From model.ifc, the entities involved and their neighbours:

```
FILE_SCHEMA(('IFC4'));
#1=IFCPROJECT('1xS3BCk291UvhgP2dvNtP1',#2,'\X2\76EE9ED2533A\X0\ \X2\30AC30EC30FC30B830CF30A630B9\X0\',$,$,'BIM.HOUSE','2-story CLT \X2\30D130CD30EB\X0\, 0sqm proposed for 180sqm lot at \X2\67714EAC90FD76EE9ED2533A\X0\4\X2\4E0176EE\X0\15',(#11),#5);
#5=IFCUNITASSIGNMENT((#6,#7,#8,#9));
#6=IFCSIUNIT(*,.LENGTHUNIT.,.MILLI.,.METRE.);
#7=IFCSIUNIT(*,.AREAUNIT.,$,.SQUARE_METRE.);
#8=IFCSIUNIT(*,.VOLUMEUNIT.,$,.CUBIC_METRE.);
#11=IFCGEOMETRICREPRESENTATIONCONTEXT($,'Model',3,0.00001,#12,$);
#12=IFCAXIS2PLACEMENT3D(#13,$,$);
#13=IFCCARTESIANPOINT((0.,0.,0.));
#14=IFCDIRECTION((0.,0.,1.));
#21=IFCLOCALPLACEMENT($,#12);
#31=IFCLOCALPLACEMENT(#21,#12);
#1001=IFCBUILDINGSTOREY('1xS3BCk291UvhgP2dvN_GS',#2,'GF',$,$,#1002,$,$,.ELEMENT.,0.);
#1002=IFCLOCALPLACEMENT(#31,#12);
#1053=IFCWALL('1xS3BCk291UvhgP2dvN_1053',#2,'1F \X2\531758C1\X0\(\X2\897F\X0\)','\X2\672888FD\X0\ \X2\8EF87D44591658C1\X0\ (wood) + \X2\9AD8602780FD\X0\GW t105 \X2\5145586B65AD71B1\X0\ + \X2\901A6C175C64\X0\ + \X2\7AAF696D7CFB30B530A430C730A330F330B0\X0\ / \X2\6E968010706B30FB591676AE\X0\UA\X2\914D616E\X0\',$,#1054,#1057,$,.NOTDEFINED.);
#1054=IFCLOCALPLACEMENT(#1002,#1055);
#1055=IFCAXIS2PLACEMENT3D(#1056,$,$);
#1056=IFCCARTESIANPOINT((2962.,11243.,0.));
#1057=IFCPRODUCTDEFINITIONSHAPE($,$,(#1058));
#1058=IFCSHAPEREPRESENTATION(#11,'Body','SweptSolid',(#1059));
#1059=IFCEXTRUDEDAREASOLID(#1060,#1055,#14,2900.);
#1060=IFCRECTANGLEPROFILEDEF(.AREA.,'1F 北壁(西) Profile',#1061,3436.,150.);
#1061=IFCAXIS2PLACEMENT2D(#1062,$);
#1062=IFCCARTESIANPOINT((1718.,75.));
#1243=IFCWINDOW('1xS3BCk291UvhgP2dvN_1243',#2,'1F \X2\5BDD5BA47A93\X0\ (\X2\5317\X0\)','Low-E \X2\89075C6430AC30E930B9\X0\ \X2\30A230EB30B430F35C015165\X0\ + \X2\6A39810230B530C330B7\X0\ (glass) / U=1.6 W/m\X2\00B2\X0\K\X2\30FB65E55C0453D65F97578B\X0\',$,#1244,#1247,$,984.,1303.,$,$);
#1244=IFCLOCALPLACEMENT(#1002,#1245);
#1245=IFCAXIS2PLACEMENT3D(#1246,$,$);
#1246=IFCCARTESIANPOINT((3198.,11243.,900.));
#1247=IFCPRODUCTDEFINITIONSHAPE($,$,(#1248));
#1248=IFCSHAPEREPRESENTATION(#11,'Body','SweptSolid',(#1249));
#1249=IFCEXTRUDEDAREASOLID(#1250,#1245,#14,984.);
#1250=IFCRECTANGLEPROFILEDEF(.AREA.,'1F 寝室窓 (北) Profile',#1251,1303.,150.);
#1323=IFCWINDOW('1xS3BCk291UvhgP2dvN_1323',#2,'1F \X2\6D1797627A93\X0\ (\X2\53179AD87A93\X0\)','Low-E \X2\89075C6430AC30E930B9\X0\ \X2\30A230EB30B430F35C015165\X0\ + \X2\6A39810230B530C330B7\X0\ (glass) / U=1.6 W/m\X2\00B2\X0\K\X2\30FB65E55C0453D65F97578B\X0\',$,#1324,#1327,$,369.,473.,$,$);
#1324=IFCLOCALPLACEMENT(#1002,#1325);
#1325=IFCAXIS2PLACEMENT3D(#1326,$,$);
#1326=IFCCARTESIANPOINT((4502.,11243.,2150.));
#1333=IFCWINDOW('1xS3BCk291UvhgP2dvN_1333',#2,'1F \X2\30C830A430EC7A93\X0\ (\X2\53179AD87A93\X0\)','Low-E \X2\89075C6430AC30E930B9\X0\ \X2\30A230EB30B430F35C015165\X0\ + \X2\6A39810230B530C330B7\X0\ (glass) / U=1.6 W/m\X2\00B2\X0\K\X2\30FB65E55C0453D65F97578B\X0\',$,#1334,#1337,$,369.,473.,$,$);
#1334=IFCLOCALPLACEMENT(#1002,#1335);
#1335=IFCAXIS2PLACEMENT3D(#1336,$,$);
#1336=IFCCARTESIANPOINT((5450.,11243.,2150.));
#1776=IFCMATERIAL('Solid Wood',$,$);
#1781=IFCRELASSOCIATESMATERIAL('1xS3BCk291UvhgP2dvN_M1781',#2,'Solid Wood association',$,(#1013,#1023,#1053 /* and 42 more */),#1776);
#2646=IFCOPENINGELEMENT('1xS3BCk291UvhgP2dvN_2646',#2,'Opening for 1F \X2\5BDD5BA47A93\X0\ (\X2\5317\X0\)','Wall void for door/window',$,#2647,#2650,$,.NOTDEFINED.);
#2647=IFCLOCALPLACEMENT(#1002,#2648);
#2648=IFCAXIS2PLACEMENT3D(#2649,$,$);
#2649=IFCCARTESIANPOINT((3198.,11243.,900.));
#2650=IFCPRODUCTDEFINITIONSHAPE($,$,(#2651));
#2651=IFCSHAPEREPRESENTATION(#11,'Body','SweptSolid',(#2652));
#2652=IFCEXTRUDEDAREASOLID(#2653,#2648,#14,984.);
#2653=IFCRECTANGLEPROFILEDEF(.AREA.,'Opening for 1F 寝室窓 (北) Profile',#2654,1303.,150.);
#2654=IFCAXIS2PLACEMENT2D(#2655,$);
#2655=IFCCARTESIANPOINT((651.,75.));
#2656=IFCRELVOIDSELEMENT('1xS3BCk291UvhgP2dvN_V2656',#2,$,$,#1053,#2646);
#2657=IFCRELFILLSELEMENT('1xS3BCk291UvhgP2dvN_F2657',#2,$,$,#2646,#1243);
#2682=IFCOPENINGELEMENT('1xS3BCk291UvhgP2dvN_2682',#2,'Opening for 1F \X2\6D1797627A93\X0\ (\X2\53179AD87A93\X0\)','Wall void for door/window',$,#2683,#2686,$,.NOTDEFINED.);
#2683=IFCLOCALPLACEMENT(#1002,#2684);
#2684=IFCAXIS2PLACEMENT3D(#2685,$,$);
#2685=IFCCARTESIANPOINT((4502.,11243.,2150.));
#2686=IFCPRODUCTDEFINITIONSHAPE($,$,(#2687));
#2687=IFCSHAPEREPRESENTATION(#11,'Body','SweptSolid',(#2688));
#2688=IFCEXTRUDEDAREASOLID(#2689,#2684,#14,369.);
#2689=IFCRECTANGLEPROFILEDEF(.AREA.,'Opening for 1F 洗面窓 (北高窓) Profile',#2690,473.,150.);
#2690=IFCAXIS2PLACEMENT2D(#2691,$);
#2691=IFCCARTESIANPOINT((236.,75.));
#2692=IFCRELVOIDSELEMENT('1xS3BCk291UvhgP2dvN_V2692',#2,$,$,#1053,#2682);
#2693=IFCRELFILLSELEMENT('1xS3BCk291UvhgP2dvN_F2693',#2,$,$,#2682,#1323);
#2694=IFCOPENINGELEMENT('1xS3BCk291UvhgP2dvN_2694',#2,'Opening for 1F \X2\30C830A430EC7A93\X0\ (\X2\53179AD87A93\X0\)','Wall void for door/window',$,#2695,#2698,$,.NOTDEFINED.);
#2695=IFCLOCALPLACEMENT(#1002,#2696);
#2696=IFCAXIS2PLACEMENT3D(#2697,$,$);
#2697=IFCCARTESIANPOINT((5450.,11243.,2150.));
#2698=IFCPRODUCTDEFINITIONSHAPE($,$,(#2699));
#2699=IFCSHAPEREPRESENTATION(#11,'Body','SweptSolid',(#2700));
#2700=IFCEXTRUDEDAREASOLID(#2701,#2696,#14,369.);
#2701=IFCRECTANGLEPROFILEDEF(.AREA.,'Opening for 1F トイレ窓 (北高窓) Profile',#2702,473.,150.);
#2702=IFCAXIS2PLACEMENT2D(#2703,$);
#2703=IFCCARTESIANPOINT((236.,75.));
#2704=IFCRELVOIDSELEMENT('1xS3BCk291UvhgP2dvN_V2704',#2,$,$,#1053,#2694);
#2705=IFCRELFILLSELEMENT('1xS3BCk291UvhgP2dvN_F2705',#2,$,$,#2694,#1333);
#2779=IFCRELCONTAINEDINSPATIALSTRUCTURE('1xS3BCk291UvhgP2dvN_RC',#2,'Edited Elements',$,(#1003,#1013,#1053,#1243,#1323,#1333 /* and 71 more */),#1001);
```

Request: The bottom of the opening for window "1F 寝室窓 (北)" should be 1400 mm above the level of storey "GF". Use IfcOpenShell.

```python
import numpy as np
import ifcopenshell
import ifcopenshell.api.geometry
import ifcopenshell.geom
import ifcopenshell.util.element
import ifcopenshell.util.placement
import ifcopenshell.util.shape
import ifcopenshell.util.unit

model = ifcopenshell.open("model.ifc")
unit_scale = ifcopenshell.util.unit.calculate_unit_scale(model)

window = model.by_guid("1xS3BCk291UvhgP2dvN_1243")
opening = window.FillsVoids[0].RelatingOpeningElement
storey = ifcopenshell.util.element.get_container(window, ifc_class="IfcBuildingStorey")
level = ifcopenshell.util.placement.get_local_placement(storey.ObjectPlacement)[2, 3]

# The opening's origin need not be at the sill, so measure its lowest point.
shape = ifcopenshell.geom.create_shape(ifcopenshell.geom.settings(), opening)
bottom = ifcopenshell.util.shape.get_shape_bottom_elevation(shape, shape.geometry) / unit_scale
dz = level + 1400.0 - bottom

shift = np.array([0.0, 0.0, dz])
# The window is not placed relative to its opening, so move both.
for product in (opening, window):
    matrix = ifcopenshell.util.placement.get_local_placement(product.ObjectPlacement)
    matrix[:3, 3] += shift
    ifcopenshell.api.geometry.edit_object_placement(model, product=product, matrix=matrix, is_si=False)

print(f"moved by {dz * unit_scale:+.3f} m")

model.write("model-out.ifc")
```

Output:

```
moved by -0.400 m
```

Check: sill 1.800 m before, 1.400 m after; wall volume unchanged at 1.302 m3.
